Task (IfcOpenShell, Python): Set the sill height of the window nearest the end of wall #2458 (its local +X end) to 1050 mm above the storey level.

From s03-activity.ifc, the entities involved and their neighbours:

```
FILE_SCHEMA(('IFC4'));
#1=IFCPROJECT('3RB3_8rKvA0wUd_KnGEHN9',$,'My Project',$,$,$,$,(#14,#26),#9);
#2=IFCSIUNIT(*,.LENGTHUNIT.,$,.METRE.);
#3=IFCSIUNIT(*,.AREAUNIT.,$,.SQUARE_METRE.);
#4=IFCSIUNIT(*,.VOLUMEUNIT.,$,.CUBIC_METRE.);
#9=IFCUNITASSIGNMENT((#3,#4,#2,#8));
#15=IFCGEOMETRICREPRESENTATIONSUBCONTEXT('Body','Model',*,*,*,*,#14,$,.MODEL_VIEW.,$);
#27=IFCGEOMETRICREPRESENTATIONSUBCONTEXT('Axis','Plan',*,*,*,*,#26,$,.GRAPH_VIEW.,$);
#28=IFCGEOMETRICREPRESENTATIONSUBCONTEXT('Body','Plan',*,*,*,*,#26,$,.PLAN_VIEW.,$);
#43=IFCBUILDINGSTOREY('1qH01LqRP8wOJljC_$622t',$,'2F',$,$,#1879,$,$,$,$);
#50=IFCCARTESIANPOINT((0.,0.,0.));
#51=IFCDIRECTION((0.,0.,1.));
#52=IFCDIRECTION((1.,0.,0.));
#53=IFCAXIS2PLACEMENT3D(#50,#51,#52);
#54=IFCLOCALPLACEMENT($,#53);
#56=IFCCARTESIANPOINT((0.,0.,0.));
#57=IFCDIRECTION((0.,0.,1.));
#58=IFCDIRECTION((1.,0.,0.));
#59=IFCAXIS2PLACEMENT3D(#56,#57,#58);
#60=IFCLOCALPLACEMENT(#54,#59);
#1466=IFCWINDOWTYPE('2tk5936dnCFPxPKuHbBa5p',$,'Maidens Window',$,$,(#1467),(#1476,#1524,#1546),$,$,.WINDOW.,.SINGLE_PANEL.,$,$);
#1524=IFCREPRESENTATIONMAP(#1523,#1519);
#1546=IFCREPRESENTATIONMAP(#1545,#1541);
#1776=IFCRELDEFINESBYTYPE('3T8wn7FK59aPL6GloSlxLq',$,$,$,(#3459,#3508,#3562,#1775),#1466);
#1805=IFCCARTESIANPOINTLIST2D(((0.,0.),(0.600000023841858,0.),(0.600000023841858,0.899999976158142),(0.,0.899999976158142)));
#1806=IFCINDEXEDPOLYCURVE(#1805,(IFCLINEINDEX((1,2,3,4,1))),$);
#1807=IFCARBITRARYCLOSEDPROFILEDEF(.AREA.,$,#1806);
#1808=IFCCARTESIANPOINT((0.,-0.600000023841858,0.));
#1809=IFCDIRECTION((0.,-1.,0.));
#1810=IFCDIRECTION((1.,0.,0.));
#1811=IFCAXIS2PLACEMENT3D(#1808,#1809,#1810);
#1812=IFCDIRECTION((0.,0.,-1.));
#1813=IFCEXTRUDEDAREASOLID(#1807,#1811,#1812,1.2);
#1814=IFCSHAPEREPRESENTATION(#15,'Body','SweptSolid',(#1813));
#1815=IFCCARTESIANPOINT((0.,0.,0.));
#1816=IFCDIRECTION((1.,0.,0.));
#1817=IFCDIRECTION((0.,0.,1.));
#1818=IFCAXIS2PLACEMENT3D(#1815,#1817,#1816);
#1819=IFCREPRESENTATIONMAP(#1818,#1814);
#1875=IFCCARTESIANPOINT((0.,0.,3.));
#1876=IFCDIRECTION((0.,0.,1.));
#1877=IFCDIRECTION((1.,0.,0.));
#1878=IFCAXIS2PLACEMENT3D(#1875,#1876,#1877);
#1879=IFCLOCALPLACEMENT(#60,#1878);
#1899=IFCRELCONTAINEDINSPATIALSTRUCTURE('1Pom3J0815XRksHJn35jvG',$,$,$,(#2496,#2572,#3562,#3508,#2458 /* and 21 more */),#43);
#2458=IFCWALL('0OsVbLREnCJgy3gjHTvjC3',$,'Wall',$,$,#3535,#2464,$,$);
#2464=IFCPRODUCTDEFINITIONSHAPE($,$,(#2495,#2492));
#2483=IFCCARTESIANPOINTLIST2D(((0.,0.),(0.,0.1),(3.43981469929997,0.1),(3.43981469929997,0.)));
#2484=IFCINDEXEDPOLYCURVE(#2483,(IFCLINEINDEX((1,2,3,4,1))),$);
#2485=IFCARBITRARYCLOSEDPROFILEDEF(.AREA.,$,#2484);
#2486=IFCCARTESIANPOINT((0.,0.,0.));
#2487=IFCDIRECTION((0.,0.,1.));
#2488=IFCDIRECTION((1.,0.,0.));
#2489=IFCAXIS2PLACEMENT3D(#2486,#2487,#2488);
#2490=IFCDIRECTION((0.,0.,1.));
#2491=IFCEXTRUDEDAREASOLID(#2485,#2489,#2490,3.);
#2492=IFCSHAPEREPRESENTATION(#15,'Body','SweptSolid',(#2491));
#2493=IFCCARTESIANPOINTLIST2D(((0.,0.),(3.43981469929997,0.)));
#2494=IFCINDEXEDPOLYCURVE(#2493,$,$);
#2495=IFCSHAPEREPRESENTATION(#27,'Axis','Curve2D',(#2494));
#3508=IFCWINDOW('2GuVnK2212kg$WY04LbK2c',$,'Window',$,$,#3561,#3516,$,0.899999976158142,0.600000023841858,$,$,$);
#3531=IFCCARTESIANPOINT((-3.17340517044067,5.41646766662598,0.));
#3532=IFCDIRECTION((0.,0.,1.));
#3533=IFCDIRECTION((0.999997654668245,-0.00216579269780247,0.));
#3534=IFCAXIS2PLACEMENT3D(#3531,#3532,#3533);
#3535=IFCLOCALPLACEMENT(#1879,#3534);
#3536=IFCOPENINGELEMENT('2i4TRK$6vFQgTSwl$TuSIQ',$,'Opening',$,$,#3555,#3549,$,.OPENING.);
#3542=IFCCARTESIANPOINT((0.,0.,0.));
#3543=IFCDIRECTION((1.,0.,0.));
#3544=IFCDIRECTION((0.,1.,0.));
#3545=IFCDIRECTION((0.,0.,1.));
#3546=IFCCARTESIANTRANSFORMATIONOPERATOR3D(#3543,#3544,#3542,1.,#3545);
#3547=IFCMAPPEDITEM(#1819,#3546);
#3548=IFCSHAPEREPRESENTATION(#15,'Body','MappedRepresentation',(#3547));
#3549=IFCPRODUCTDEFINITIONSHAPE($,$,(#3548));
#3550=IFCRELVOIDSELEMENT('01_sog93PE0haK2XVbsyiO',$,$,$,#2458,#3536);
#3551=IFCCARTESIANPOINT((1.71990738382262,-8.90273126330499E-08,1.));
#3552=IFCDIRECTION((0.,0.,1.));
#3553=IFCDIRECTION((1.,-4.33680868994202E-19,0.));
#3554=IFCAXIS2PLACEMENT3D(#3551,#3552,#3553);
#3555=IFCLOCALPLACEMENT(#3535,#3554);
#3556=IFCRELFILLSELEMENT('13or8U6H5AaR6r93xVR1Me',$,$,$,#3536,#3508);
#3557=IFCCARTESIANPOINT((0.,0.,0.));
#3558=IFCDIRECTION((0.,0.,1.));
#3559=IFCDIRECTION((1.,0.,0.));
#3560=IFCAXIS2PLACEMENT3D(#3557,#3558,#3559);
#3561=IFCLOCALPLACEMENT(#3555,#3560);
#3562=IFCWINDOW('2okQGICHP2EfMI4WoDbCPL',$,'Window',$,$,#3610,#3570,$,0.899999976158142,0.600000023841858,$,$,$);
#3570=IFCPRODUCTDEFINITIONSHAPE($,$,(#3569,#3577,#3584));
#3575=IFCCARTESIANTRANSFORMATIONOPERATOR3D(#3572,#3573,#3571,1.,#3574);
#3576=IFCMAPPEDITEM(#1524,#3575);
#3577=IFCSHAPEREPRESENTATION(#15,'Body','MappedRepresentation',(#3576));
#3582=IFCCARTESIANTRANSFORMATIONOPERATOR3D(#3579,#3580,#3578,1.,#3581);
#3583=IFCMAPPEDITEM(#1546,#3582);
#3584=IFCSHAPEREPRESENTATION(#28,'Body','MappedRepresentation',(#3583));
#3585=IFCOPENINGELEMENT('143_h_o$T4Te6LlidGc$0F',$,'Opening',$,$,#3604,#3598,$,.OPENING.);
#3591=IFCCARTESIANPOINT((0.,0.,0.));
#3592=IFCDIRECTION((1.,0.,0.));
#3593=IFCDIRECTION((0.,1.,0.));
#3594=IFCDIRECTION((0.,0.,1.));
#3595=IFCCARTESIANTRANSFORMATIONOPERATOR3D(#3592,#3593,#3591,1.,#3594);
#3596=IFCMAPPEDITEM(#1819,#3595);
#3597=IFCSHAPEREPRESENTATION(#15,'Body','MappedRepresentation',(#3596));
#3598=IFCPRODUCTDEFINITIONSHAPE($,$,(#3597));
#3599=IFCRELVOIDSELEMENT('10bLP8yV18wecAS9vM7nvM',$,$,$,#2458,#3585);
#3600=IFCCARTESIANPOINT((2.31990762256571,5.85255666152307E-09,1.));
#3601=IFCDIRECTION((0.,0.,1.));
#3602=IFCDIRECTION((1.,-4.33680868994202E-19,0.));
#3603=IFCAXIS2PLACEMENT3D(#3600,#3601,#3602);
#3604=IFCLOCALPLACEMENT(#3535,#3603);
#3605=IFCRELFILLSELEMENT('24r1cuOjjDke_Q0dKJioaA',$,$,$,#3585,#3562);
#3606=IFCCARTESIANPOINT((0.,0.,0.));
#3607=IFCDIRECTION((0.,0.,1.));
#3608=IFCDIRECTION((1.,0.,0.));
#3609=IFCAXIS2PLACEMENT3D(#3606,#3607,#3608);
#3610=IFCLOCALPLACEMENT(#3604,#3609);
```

```python
import numpy as np
import ifcopenshell
import ifcopenshell.api.geometry
import ifcopenshell.geom
import ifcopenshell.util.element
import ifcopenshell.util.placement
import ifcopenshell.util.shape
import ifcopenshell.util.unit

model = ifcopenshell.open("s03-activity.ifc")
unit_scale = ifcopenshell.util.unit.calculate_unit_scale(model)

window = model.by_guid("2okQGICHP2EfMI4WoDbCPL")
opening = window.FillsVoids[0].RelatingOpeningElement
storey = ifcopenshell.util.element.get_container(window, ifc_class="IfcBuildingStorey")
level = ifcopenshell.util.placement.get_local_placement(storey.ObjectPlacement)[2, 3]

# The opening's origin need not be at the sill, so measure its lowest point.
shape = ifcopenshell.geom.create_shape(ifcopenshell.geom.settings(), opening)
bottom = ifcopenshell.util.shape.get_shape_bottom_elevation(shape, shape.geometry) / unit_scale
dz = level + 1.05 / unit_scale - bottom

shift = np.array([0.0, 0.0, dz])
# The window is placed relative to its opening, so it follows when the opening moves.
matrix = ifcopenshell.util.placement.get_local_placement(opening.ObjectPlacement)
matrix[:3, 3] += shift
ifcopenshell.api.geometry.edit_object_placement(
    model, product=opening, matrix=matrix, is_si=False, should_transform_children=True
)

print(f"moved by {dz * unit_scale:+.3f} m")

model.write("s03-activity_v2.ifc")
```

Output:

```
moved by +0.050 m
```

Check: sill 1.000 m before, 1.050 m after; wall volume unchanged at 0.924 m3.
